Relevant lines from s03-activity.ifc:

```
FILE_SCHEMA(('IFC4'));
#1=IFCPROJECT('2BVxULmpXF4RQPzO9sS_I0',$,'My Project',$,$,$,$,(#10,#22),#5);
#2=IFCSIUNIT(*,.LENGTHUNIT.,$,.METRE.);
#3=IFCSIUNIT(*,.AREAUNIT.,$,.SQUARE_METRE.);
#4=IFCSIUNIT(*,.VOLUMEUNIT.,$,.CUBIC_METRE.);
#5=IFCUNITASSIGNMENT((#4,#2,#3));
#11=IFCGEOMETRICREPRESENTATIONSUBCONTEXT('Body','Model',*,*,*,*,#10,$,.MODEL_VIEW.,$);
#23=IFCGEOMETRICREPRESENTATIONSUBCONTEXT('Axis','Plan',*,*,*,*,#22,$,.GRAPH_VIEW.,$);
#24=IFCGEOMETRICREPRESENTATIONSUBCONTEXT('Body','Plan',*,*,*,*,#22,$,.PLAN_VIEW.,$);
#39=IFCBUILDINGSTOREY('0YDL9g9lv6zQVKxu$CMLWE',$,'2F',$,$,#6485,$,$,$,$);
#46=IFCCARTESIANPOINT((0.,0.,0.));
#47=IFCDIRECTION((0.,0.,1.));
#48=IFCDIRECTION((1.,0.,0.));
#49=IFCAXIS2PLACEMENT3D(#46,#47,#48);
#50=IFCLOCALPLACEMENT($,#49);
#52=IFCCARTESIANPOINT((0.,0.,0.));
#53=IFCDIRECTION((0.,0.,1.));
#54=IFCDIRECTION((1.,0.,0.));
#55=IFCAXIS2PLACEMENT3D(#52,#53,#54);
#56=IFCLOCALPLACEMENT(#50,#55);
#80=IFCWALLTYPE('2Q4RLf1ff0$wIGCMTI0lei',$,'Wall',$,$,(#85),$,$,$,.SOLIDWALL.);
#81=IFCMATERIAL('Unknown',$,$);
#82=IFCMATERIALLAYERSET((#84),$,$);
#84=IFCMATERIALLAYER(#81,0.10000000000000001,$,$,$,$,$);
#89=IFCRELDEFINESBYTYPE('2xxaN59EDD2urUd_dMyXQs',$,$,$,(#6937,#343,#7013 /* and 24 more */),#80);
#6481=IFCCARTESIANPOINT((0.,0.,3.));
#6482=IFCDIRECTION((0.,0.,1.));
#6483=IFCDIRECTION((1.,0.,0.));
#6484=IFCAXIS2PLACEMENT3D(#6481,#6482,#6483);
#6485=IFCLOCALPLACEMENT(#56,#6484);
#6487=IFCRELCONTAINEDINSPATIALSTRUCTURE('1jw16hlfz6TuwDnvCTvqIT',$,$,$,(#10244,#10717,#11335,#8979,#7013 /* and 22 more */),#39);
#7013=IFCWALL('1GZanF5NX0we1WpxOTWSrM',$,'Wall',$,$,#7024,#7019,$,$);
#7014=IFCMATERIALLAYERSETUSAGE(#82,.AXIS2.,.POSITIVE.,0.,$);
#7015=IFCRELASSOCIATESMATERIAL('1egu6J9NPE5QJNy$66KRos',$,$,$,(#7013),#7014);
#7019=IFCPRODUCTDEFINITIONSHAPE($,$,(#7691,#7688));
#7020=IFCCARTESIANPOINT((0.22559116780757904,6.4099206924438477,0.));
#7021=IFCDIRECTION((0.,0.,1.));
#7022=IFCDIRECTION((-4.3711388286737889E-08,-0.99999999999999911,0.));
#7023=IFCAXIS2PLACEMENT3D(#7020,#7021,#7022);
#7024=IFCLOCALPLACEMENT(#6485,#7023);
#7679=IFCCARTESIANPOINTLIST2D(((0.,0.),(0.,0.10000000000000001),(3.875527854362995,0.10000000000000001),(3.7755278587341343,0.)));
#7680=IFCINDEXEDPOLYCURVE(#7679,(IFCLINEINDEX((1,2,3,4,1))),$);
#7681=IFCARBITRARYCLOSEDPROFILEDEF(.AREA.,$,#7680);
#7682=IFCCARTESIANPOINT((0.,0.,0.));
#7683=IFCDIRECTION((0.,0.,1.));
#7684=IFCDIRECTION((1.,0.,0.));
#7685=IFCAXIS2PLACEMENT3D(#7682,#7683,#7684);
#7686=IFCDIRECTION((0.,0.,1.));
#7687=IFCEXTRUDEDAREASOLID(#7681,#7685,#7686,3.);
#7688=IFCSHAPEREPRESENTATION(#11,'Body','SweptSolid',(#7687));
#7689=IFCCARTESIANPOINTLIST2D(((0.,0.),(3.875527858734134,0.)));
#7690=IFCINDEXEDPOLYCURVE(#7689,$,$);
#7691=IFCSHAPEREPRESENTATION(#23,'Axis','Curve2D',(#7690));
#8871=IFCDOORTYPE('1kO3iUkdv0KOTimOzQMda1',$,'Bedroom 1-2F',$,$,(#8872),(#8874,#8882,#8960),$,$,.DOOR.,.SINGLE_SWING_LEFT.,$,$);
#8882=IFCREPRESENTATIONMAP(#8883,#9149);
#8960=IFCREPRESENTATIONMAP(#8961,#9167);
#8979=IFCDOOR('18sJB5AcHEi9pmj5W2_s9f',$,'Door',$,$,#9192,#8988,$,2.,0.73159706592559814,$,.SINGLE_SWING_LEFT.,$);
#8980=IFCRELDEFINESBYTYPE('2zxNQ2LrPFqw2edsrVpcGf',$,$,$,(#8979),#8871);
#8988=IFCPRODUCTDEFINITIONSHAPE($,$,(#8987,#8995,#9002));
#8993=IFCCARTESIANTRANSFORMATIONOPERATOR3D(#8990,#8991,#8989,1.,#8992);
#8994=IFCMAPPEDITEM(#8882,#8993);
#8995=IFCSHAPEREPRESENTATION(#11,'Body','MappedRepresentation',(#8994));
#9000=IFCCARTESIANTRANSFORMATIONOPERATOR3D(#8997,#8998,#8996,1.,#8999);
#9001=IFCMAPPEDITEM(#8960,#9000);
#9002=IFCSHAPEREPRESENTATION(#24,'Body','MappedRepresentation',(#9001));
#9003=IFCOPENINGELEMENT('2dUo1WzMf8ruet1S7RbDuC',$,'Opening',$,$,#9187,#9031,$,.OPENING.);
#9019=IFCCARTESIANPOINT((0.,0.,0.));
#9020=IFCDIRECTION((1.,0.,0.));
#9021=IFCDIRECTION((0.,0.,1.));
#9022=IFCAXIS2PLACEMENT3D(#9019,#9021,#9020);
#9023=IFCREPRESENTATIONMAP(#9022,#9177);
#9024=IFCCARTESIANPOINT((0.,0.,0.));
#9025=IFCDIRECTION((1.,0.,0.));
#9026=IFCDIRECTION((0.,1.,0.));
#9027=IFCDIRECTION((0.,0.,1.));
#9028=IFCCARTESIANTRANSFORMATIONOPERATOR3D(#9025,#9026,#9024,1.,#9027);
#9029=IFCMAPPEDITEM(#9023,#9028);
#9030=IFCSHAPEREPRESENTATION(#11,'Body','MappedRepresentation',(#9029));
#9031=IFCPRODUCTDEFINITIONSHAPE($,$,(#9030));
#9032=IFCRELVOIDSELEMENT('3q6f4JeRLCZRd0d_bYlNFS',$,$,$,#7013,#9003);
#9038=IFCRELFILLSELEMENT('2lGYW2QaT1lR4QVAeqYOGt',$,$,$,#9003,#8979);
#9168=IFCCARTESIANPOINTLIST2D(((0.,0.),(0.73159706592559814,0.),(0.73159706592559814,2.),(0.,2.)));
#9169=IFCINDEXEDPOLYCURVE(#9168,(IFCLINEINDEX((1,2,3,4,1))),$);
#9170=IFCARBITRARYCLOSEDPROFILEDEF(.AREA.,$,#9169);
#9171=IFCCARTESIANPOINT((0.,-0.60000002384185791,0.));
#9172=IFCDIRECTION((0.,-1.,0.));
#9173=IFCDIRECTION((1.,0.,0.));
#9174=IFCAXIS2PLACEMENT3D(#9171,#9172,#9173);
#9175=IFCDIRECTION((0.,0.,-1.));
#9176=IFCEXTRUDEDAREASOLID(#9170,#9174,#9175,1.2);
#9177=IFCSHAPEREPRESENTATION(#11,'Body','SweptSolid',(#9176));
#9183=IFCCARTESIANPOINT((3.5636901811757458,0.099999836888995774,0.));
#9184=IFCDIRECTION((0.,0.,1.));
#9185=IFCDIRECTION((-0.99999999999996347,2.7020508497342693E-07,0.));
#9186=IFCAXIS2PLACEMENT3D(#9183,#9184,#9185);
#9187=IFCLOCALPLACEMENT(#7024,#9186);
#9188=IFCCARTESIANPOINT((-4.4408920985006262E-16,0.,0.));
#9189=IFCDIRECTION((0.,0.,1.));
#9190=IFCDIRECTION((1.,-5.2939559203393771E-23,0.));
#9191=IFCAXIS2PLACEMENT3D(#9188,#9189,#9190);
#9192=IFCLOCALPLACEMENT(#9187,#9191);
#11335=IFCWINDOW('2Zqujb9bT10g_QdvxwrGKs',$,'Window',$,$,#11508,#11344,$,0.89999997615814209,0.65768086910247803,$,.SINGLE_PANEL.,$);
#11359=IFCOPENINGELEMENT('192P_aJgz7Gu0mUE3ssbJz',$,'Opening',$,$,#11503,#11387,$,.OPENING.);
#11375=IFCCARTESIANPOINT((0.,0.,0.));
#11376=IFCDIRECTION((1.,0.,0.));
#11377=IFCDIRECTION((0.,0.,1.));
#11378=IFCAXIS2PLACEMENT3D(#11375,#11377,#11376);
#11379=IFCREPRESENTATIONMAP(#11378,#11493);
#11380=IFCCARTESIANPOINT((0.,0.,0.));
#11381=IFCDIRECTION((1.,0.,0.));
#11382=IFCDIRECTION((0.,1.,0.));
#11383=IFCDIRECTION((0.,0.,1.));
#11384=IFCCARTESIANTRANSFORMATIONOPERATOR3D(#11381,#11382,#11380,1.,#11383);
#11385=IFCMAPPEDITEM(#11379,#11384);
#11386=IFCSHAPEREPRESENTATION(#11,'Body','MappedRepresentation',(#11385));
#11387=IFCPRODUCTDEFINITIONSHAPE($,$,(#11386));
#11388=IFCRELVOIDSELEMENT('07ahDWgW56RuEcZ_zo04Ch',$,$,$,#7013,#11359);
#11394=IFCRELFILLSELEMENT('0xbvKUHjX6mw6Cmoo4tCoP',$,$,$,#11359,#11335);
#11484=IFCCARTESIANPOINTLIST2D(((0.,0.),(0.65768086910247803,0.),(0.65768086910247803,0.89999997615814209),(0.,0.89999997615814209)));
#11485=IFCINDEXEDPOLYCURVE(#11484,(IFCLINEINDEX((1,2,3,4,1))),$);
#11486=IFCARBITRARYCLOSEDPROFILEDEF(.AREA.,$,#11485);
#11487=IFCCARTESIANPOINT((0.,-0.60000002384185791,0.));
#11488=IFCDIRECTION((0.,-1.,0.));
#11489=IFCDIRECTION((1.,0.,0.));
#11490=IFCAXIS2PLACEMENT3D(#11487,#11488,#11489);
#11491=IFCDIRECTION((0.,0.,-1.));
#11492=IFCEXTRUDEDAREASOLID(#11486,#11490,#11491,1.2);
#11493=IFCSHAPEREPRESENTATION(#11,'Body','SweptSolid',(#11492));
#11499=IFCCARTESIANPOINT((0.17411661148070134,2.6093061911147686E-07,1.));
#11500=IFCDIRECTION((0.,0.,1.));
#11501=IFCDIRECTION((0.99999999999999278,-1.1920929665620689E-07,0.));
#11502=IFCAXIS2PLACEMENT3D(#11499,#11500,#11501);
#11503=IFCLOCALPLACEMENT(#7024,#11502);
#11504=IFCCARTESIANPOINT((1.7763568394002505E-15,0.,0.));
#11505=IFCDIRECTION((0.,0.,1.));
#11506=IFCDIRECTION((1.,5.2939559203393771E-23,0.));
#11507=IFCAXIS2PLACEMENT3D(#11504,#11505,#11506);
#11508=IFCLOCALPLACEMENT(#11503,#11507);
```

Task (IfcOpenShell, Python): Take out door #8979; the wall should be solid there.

```python
import ifcopenshell
import ifcopenshell.api.feature
import ifcopenshell.api.root
import ifcopenshell.geom
import ifcopenshell.util.shape

model = ifcopenshell.open("s03-activity.ifc")
settings = ifcopenshell.geom.settings()


def volume(element):
    """Net volume in cubic metres, openings subtracted."""
    shape = ifcopenshell.geom.create_shape(settings, element)
    return ifcopenshell.util.shape.get_volume(shape.geometry)


door = model.by_id(8979)
opening = door.FillsVoids[0].RelatingOpeningElement
wall = opening.VoidsElements[0].RelatingBuildingElement
before = volume(wall)

ifcopenshell.api.root.remove_product(model, product=door)
ifcopenshell.api.feature.remove_feature(model, feature=opening)

after = volume(wall)

print(f"wall volume {before:.3f} -> {after:.3f} m3")

model.write("s03-activity-out.ifc")
```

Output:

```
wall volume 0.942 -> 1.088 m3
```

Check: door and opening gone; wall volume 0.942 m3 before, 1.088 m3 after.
